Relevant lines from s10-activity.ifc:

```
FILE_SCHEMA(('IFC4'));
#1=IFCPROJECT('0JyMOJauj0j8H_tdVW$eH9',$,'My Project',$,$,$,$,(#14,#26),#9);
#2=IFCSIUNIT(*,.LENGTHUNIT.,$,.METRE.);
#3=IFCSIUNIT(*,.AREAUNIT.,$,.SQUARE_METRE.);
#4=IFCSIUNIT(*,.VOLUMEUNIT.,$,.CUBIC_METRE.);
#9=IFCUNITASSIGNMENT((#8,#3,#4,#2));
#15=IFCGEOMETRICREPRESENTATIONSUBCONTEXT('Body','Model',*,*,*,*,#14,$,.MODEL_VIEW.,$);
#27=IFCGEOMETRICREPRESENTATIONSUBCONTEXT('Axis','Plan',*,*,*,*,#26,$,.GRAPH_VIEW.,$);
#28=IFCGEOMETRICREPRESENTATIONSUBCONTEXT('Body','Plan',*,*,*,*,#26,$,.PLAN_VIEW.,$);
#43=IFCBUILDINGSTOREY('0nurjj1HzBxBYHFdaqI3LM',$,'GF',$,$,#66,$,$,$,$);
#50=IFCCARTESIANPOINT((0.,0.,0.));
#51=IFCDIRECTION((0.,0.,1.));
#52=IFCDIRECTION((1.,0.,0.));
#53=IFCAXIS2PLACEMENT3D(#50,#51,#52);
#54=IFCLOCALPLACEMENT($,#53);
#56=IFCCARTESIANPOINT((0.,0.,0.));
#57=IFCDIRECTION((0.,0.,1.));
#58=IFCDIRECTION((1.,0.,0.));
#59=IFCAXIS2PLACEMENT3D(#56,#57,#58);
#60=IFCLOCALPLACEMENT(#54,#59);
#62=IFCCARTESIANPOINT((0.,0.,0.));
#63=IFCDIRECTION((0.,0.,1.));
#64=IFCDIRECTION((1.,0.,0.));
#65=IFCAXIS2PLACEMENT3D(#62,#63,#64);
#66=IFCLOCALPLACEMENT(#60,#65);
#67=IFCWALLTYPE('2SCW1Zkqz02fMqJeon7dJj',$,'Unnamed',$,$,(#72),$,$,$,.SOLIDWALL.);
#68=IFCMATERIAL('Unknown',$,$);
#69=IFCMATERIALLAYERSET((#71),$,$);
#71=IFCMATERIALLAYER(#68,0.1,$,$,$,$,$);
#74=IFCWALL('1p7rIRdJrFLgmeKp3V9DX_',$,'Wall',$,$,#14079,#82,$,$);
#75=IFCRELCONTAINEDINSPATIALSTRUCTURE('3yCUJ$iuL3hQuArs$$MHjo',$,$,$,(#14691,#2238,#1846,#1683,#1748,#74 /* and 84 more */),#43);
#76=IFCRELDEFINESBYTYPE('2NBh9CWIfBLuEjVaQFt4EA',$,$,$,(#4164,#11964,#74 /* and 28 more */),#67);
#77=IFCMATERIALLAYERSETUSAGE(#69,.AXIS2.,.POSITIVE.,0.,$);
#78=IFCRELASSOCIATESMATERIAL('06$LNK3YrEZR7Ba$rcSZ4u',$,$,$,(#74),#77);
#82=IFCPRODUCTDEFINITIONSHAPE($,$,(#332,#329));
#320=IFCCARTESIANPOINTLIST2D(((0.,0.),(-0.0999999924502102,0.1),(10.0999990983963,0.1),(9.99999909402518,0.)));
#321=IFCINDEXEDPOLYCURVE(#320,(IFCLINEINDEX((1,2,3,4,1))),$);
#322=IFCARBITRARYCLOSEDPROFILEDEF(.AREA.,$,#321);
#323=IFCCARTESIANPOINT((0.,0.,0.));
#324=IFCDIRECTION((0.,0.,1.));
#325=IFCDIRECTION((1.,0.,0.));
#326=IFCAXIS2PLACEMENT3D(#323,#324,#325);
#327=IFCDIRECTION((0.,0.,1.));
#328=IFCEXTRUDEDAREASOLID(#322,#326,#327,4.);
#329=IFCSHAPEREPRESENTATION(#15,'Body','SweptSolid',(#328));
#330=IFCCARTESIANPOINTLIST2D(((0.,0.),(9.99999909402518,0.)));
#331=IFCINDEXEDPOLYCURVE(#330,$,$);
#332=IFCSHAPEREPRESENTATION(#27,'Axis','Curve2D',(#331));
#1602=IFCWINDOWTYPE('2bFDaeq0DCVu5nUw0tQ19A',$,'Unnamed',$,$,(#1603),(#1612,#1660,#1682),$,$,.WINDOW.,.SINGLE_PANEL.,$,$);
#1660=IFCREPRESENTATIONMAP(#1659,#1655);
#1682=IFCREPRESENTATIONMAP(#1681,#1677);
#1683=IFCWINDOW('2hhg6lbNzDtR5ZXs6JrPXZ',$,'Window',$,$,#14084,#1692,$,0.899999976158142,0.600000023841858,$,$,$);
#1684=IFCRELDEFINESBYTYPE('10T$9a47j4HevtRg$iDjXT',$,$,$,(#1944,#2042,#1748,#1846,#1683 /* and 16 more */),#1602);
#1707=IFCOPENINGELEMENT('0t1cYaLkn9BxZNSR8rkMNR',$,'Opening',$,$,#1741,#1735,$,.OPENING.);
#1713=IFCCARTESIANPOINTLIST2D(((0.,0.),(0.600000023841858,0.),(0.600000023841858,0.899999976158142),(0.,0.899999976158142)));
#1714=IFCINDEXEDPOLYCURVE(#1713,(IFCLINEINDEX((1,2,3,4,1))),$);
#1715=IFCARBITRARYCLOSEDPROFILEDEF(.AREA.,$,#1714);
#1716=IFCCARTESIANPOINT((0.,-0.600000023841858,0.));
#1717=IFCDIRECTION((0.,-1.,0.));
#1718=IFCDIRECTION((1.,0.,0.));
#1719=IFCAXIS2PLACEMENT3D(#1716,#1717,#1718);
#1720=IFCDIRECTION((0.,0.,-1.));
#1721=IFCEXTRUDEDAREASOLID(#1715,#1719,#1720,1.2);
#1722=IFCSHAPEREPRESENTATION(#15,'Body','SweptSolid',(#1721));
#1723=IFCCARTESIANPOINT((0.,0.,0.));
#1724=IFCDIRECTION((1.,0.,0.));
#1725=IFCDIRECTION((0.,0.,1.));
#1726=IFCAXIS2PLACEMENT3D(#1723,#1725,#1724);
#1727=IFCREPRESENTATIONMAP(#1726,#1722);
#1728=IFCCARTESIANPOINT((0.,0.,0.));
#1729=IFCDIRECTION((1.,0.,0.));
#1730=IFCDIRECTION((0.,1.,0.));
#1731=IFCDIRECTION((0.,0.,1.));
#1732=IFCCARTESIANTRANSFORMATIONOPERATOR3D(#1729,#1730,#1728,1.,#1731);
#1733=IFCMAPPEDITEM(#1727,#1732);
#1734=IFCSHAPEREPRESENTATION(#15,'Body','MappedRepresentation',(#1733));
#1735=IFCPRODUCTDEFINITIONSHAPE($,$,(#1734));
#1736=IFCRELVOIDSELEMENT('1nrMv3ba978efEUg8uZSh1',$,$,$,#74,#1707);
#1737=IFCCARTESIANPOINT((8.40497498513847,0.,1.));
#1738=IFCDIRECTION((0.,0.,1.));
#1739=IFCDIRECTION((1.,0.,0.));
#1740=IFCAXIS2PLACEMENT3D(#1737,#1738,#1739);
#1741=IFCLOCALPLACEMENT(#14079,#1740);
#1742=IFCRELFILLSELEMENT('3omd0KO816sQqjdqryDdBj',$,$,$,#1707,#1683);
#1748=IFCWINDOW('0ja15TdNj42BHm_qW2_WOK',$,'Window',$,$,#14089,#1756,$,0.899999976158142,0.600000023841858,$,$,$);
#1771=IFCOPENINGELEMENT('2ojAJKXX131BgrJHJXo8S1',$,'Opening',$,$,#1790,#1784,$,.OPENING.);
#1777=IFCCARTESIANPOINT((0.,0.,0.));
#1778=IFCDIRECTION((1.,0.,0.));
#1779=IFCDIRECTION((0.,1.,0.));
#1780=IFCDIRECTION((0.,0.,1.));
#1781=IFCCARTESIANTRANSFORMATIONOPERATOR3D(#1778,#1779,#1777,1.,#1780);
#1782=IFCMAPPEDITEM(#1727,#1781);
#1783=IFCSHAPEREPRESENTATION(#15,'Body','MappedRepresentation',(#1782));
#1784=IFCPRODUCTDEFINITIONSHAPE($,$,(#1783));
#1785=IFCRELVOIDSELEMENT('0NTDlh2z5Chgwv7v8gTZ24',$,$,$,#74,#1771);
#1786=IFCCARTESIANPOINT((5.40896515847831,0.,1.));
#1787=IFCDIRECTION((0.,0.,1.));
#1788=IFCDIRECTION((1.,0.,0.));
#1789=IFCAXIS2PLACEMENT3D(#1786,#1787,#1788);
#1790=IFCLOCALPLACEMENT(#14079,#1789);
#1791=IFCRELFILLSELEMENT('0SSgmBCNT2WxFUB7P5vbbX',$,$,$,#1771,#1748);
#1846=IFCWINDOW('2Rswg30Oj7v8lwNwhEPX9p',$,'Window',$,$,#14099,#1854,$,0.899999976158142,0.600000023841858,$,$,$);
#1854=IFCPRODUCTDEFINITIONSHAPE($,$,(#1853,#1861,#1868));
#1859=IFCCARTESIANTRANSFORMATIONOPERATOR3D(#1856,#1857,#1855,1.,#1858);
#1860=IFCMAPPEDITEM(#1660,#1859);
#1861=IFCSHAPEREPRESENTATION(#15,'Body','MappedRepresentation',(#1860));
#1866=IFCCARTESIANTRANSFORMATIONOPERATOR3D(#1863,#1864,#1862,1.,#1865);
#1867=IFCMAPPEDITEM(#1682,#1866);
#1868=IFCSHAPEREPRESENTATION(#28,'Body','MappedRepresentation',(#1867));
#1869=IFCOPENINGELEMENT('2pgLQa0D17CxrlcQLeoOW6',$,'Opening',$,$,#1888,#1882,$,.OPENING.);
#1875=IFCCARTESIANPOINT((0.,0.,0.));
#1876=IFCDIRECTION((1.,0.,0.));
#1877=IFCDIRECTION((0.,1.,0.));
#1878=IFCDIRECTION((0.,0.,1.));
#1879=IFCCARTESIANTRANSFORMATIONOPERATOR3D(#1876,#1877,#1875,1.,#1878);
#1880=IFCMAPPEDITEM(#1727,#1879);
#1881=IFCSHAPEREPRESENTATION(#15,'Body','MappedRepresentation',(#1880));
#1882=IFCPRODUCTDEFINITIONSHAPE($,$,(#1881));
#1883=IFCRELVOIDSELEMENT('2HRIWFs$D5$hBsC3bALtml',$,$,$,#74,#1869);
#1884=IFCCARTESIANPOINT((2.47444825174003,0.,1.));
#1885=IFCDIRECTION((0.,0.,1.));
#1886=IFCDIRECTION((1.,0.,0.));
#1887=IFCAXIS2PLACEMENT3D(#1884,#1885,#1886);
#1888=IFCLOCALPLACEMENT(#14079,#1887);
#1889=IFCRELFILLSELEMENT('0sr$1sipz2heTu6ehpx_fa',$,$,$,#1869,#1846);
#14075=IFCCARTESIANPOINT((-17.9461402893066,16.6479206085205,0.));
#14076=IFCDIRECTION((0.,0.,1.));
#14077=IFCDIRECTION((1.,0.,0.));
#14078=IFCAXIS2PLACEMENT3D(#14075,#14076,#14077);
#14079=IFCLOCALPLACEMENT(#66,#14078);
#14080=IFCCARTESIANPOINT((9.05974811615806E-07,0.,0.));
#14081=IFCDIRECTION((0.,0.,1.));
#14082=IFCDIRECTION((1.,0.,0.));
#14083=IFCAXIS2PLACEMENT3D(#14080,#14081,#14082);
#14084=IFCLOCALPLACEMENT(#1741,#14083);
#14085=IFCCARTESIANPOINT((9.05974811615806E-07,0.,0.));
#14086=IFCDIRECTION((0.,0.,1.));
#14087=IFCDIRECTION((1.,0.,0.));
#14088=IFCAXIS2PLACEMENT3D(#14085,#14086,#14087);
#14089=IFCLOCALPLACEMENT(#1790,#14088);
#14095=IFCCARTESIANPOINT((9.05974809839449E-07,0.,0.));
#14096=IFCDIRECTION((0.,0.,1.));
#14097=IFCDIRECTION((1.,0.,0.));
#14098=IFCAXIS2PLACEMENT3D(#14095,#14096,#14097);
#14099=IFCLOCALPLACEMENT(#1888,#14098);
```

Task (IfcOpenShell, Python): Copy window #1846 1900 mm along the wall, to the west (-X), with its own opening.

```python
import ifcopenshell
import ifcopenshell.api.feature
import ifcopenshell.api.geometry
import ifcopenshell.api.root
import ifcopenshell.geom
import ifcopenshell.util.element
import ifcopenshell.util.placement
import ifcopenshell.util.shape
import ifcopenshell.util.unit

model = ifcopenshell.open("s10-activity.ifc")
unit_scale = ifcopenshell.util.unit.calculate_unit_scale(model)
settings = ifcopenshell.geom.settings()


def volume(element):
    """Net volume in cubic metres, openings subtracted."""
    shape = ifcopenshell.geom.create_shape(settings, element)
    return ifcopenshell.util.shape.get_volume(shape.geometry)


window = model.by_id(1846)
opening = window.FillsVoids[0].RelatingOpeningElement
wall = opening.VoidsElements[0].RelatingBuildingElement
before = volume(wall)
shift = ifcopenshell.util.placement.get_local_placement(wall.ObjectPlacement)[:3, 0] * -1.9 / unit_scale

# copy_class copies the void relationship, type, container and properties, but no geometry.
new_opening = ifcopenshell.api.root.copy_class(model, product=opening)
new_opening.Representation = ifcopenshell.util.element.copy_deep(
    model, opening.Representation, exclude=["IfcGeometricRepresentationContext", "IfcRepresentationMap"]
)
new_window = ifcopenshell.api.root.copy_class(model, product=window)
new_window.Representation = ifcopenshell.util.element.copy_deep(
    model, window.Representation, exclude=["IfcGeometricRepresentationContext", "IfcRepresentationMap"]
)
ifcopenshell.api.feature.add_filling(model, opening=new_opening, element=new_window)

for old, new in ((opening, new_opening), (window, new_window)):
    matrix = ifcopenshell.util.placement.get_local_placement(old.ObjectPlacement)
    matrix[:3, 3] += shift
    ifcopenshell.api.geometry.edit_object_placement(model, product=new, matrix=matrix, is_si=False)

after = volume(wall)

print(f"wall volume {before:.3f} -> {after:.3f} m3")

model.write("s10-activity_rev.ifc")
```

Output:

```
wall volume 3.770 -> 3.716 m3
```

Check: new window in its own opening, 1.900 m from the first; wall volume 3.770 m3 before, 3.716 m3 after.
